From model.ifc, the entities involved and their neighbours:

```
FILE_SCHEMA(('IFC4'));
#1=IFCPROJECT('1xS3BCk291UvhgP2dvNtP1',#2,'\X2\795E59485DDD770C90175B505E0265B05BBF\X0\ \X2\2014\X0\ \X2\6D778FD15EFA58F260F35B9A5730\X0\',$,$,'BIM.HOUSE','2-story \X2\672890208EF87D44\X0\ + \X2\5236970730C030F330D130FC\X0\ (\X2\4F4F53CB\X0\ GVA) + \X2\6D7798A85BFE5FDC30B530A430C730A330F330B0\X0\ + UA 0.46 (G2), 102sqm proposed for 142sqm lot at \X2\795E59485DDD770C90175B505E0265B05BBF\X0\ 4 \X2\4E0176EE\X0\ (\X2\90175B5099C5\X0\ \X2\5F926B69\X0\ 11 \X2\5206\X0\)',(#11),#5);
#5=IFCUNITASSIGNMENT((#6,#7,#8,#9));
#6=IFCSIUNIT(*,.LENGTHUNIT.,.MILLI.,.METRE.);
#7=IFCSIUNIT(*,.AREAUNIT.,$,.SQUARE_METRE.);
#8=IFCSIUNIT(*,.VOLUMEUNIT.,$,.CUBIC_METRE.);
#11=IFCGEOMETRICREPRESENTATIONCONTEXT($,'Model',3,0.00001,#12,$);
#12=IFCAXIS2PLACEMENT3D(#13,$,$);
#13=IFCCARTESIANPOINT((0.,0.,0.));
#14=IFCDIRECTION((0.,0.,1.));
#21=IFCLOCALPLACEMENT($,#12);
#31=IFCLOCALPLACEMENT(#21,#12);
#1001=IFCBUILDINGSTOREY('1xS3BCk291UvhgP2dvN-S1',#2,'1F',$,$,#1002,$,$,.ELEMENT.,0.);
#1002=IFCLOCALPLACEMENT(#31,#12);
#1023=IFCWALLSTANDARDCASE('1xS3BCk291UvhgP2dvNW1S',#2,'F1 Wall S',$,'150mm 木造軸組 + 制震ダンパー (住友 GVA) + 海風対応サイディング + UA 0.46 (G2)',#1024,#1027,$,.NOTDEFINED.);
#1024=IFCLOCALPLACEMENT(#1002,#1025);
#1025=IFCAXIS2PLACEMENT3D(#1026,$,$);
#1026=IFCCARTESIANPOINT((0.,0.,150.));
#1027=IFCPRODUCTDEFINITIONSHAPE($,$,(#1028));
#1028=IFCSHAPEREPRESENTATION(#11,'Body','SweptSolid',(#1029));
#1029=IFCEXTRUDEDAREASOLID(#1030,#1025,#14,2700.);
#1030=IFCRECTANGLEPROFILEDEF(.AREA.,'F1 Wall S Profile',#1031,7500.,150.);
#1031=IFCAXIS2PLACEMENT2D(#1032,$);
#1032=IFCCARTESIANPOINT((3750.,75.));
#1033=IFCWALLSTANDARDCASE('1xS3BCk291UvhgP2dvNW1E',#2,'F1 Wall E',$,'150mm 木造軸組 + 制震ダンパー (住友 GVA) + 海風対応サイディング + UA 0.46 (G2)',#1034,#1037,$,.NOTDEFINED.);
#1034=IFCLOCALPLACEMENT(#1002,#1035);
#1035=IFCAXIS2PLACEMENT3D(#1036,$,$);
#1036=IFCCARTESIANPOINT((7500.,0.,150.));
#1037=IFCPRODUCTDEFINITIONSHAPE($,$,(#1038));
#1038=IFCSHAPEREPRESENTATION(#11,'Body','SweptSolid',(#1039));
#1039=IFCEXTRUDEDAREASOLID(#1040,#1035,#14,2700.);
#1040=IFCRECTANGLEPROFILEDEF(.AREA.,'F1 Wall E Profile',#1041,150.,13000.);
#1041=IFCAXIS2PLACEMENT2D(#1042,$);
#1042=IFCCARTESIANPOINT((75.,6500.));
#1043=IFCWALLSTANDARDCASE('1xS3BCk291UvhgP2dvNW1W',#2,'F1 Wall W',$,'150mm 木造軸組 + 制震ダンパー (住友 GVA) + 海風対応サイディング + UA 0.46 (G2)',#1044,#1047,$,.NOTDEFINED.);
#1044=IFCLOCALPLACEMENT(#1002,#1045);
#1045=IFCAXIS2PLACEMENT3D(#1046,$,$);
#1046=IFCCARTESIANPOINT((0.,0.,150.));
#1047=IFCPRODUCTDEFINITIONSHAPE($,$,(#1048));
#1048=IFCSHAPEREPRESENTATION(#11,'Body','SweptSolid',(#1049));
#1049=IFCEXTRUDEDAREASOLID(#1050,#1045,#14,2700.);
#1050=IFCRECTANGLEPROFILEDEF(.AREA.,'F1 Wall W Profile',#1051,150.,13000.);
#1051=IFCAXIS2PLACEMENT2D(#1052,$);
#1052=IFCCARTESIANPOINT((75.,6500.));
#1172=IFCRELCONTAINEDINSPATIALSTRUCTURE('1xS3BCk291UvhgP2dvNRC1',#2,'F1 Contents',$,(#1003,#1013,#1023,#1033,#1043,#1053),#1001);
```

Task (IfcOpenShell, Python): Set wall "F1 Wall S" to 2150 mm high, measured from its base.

```python
import ifcopenshell
import ifcopenshell.geom
import ifcopenshell.util.shape

model = ifcopenshell.open("model.ifc")
settings = ifcopenshell.geom.settings()


def volume(element):
    """Net volume in cubic metres, openings subtracted."""
    shape = ifcopenshell.geom.create_shape(settings, element)
    return ifcopenshell.util.shape.get_volume(shape.geometry)


wall = model.by_guid("1xS3BCk291UvhgP2dvNW1S")
before = volume(wall)

body = next(r for r in wall.Representation.Representations if r.RepresentationIdentifier == "Body")
solid = body.Items[0]
old_height = solid.Depth
solid.Depth = 2150.0
after = volume(wall)

print(f"height {old_height:g} -> {solid.Depth:g}, volume {before:.3f} -> {after:.3f} m3")

model.write("model_v2.ifc")
```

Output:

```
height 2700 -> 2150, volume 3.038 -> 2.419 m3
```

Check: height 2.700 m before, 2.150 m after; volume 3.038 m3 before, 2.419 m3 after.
